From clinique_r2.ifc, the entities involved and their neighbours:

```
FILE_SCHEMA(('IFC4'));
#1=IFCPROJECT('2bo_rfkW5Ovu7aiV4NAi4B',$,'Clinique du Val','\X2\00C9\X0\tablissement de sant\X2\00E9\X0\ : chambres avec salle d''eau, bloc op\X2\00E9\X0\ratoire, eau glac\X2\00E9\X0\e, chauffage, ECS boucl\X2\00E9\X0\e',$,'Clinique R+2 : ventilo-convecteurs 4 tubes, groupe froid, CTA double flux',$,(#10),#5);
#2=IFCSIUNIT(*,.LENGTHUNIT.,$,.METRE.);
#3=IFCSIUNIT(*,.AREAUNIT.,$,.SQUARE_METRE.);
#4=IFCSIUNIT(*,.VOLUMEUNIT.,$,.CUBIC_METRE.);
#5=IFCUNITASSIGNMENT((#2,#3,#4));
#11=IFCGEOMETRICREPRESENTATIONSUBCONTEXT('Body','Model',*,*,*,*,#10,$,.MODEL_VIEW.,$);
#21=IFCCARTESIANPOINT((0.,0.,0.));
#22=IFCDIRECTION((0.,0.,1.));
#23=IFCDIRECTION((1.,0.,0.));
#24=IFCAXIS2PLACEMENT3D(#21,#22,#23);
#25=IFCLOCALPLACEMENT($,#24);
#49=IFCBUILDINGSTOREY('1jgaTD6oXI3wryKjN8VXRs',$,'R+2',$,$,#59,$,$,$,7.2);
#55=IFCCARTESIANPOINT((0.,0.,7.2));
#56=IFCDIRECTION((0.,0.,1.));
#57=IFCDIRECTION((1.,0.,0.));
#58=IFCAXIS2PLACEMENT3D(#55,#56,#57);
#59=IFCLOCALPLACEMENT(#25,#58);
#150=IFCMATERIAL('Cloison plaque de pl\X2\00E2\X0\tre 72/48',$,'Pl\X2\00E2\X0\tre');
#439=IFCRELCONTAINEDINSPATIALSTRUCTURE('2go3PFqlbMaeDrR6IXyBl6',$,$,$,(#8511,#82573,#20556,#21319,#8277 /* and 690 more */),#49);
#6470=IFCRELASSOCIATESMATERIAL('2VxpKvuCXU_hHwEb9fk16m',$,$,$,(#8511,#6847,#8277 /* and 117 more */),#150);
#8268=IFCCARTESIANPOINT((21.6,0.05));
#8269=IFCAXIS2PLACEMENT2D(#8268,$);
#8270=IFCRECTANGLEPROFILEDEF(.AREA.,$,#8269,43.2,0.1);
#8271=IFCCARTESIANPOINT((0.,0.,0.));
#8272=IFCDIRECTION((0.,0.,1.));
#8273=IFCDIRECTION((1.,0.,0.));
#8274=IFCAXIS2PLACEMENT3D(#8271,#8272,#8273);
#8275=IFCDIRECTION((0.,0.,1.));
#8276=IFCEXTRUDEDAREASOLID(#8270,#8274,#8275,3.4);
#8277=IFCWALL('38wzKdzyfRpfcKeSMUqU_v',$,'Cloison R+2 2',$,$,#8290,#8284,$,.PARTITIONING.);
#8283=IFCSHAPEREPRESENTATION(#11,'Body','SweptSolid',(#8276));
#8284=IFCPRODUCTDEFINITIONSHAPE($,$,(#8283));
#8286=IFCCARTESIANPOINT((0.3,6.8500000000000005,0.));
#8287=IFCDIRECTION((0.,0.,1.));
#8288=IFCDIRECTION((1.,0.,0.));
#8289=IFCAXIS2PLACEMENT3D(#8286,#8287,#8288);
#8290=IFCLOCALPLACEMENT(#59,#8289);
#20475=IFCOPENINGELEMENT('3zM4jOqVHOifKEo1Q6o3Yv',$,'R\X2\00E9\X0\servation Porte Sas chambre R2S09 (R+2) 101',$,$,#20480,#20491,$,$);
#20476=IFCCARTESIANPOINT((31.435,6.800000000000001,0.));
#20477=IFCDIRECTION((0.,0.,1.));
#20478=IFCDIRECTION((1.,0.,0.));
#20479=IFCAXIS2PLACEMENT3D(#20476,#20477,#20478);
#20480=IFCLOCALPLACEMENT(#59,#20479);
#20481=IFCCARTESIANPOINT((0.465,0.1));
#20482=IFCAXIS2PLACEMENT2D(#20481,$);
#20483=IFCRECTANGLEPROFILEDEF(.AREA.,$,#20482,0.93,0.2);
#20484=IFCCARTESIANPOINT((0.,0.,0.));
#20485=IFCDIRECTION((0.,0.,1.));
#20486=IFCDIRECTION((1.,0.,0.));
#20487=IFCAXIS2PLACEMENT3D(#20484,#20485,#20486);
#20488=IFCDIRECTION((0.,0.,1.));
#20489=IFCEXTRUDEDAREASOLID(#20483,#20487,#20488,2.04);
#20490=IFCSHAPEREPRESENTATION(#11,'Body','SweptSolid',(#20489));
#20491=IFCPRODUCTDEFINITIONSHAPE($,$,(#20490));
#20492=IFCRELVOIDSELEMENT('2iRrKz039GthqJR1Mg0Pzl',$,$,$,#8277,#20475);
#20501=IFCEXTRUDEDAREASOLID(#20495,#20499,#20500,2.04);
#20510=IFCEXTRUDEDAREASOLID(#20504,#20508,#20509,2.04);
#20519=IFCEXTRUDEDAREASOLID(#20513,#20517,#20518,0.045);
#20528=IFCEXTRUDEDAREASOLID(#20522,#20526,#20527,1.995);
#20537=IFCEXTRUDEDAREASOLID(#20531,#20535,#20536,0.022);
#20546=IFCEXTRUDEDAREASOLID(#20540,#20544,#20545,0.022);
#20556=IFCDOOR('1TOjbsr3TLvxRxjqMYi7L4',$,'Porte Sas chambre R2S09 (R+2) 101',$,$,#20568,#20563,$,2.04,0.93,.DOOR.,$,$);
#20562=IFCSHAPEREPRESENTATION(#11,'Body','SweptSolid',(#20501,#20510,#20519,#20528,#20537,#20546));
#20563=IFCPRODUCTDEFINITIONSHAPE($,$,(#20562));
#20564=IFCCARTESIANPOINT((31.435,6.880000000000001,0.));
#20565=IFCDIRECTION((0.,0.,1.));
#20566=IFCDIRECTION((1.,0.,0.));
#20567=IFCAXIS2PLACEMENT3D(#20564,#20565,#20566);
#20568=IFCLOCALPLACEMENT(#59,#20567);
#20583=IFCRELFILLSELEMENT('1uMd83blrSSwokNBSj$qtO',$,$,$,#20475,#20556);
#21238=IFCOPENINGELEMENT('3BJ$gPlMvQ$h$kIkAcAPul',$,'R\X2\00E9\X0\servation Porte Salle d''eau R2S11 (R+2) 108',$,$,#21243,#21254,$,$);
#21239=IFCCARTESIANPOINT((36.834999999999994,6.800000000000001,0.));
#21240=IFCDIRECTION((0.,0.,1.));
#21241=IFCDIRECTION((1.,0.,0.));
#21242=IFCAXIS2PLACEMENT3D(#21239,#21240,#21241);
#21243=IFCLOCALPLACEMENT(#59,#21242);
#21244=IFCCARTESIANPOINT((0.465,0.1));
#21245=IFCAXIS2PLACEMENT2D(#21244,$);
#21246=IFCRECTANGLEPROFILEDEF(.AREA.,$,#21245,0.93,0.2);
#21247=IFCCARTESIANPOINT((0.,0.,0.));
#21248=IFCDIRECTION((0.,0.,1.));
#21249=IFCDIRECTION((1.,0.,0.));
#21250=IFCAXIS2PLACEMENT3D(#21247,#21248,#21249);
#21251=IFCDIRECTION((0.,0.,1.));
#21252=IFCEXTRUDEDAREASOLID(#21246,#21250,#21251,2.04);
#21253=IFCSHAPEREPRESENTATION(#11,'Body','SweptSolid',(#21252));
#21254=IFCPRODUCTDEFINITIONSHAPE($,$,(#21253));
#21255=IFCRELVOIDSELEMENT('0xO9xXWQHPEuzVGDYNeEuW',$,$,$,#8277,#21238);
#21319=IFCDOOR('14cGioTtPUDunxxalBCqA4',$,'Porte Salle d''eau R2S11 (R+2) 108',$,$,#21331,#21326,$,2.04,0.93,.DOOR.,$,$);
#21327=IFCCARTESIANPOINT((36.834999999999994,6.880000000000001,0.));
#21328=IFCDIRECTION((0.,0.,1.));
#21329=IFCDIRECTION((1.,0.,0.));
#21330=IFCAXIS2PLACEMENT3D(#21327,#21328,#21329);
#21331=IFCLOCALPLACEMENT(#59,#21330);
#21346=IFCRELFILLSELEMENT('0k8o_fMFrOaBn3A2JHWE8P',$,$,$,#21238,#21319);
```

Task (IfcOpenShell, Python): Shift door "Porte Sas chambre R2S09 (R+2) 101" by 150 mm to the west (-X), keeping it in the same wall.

```python
import ifcopenshell
import ifcopenshell.api.geometry
import ifcopenshell.util.placement

model = ifcopenshell.open("clinique_r2.ifc")

door = model.by_guid("1TOjbsr3TLvxRxjqMYi7L4")
opening = door.FillsVoids[0].RelatingOpeningElement
wall = opening.VoidsElements[0].RelatingBuildingElement

wall_matrix = ifcopenshell.util.placement.get_local_placement(wall.ObjectPlacement)
shift = wall_matrix[:3, 0] * -0.15
before = ifcopenshell.util.placement.get_local_placement(door.ObjectPlacement)[:3, 3].copy()

# The door is not placed relative to its opening, so move both.
for product in (opening, door):
    matrix = ifcopenshell.util.placement.get_local_placement(product.ObjectPlacement)
    matrix[:3, 3] += shift
    ifcopenshell.api.geometry.edit_object_placement(model, product=product, matrix=matrix, is_si=False)

after = ifcopenshell.util.placement.get_local_placement(door.ObjectPlacement)[:3, 3]
print("door moved by", (after - before).round(3) + 0.0)

model.write("clinique_r2_v2.ifc")
```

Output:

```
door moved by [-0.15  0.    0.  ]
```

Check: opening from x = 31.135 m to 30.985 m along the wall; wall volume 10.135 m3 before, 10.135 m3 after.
